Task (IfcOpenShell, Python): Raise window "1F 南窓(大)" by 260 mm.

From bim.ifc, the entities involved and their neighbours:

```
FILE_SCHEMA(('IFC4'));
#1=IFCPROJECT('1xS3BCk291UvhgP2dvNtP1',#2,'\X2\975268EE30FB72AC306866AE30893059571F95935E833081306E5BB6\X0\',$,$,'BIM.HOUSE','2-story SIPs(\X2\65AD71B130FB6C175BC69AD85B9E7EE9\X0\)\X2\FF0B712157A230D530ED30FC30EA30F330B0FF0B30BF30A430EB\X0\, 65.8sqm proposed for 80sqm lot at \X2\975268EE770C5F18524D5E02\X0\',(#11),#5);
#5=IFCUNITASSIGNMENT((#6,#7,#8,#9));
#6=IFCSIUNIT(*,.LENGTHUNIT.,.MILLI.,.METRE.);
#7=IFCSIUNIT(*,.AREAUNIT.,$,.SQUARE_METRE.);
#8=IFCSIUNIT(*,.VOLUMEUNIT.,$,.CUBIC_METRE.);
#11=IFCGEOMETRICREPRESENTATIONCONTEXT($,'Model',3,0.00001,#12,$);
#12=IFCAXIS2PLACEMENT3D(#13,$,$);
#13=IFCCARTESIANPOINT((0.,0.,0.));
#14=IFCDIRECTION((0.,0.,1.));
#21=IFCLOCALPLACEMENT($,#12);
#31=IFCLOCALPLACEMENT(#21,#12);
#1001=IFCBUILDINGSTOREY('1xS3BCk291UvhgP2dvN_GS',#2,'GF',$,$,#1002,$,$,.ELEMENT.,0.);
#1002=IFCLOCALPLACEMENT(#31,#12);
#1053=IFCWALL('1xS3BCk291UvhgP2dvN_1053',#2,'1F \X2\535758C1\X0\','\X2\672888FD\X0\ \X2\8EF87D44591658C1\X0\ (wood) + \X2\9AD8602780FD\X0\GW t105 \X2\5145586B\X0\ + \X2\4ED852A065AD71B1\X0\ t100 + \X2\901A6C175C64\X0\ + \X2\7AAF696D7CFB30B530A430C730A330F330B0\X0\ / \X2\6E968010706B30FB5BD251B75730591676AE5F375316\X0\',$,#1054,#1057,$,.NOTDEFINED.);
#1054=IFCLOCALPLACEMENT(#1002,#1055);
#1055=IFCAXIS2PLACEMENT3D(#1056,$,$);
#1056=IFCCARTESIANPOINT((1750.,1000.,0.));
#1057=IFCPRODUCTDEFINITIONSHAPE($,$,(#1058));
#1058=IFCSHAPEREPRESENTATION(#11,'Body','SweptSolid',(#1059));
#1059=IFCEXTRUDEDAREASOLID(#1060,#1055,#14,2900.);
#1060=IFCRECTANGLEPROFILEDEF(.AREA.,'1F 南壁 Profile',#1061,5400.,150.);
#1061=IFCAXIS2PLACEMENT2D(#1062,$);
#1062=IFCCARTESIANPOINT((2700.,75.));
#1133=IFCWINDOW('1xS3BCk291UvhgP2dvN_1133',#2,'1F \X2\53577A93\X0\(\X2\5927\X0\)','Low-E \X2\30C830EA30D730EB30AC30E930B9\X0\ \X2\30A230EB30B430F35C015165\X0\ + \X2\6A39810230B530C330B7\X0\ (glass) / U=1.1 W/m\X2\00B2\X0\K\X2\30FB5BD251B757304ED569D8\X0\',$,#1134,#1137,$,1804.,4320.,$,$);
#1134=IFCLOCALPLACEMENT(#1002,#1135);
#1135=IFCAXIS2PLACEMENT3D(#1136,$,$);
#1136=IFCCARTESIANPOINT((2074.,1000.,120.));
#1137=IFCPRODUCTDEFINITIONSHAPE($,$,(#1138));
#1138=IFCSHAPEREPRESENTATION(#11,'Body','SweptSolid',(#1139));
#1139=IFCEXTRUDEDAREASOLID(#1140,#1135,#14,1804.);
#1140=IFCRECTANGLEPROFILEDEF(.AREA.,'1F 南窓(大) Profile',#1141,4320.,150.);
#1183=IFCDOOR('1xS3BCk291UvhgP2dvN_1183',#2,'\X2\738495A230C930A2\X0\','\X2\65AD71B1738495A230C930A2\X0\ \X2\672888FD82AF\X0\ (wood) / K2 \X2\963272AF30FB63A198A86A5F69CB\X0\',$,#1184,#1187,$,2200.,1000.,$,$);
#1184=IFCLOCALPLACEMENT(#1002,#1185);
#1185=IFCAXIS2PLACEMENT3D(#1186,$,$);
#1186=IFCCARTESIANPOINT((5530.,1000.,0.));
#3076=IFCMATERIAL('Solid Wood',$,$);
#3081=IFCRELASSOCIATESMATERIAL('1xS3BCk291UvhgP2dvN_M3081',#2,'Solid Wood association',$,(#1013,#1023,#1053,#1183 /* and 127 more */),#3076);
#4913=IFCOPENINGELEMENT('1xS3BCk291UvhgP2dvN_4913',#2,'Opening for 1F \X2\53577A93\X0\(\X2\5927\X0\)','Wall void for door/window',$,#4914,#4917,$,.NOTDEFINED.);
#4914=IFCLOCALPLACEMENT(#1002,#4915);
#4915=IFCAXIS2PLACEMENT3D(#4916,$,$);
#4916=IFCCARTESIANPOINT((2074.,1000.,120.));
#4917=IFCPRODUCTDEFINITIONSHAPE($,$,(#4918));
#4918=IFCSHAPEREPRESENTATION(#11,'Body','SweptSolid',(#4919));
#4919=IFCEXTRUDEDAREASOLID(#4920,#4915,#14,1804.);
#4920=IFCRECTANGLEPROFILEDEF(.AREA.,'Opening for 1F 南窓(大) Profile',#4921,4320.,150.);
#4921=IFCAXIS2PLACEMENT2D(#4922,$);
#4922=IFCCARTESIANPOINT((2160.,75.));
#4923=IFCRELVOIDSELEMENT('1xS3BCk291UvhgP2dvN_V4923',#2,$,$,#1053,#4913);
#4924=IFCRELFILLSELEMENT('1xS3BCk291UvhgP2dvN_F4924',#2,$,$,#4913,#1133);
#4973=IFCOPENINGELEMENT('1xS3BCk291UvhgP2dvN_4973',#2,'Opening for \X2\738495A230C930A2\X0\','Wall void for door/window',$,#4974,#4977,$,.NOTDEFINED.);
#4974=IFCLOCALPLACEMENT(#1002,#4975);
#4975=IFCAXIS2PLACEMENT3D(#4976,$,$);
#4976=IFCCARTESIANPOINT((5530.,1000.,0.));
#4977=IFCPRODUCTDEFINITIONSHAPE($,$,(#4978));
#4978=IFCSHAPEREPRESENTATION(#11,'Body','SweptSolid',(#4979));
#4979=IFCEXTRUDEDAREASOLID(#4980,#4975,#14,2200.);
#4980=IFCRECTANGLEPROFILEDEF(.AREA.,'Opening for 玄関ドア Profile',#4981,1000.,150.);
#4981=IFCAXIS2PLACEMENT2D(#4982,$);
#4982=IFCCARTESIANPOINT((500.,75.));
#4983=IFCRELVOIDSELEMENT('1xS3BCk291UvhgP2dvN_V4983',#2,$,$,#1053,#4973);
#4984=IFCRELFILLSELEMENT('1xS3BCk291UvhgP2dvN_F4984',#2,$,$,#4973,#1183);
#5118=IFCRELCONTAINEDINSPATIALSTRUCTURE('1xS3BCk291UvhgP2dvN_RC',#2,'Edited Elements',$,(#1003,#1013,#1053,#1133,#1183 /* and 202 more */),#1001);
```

```python
import numpy as np
import ifcopenshell
import ifcopenshell.api.geometry
import ifcopenshell.util.placement
import ifcopenshell.util.unit

model = ifcopenshell.open("bim.ifc")
unit_scale = ifcopenshell.util.unit.calculate_unit_scale(model)

window = model.by_guid("1xS3BCk291UvhgP2dvN_1133")
opening = window.FillsVoids[0].RelatingOpeningElement
dz = 260.0

shift = np.array([0.0, 0.0, dz])
# The window is not placed relative to its opening, so move both.
for product in (opening, window):
    matrix = ifcopenshell.util.placement.get_local_placement(product.ObjectPlacement)
    matrix[:3, 3] += shift
    ifcopenshell.api.geometry.edit_object_placement(model, product=product, matrix=matrix, is_si=False)

print(f"moved by {dz * unit_scale:+.3f} m")

model.write("bim_rev.ifc")
```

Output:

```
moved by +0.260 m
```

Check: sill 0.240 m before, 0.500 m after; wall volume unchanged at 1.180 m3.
